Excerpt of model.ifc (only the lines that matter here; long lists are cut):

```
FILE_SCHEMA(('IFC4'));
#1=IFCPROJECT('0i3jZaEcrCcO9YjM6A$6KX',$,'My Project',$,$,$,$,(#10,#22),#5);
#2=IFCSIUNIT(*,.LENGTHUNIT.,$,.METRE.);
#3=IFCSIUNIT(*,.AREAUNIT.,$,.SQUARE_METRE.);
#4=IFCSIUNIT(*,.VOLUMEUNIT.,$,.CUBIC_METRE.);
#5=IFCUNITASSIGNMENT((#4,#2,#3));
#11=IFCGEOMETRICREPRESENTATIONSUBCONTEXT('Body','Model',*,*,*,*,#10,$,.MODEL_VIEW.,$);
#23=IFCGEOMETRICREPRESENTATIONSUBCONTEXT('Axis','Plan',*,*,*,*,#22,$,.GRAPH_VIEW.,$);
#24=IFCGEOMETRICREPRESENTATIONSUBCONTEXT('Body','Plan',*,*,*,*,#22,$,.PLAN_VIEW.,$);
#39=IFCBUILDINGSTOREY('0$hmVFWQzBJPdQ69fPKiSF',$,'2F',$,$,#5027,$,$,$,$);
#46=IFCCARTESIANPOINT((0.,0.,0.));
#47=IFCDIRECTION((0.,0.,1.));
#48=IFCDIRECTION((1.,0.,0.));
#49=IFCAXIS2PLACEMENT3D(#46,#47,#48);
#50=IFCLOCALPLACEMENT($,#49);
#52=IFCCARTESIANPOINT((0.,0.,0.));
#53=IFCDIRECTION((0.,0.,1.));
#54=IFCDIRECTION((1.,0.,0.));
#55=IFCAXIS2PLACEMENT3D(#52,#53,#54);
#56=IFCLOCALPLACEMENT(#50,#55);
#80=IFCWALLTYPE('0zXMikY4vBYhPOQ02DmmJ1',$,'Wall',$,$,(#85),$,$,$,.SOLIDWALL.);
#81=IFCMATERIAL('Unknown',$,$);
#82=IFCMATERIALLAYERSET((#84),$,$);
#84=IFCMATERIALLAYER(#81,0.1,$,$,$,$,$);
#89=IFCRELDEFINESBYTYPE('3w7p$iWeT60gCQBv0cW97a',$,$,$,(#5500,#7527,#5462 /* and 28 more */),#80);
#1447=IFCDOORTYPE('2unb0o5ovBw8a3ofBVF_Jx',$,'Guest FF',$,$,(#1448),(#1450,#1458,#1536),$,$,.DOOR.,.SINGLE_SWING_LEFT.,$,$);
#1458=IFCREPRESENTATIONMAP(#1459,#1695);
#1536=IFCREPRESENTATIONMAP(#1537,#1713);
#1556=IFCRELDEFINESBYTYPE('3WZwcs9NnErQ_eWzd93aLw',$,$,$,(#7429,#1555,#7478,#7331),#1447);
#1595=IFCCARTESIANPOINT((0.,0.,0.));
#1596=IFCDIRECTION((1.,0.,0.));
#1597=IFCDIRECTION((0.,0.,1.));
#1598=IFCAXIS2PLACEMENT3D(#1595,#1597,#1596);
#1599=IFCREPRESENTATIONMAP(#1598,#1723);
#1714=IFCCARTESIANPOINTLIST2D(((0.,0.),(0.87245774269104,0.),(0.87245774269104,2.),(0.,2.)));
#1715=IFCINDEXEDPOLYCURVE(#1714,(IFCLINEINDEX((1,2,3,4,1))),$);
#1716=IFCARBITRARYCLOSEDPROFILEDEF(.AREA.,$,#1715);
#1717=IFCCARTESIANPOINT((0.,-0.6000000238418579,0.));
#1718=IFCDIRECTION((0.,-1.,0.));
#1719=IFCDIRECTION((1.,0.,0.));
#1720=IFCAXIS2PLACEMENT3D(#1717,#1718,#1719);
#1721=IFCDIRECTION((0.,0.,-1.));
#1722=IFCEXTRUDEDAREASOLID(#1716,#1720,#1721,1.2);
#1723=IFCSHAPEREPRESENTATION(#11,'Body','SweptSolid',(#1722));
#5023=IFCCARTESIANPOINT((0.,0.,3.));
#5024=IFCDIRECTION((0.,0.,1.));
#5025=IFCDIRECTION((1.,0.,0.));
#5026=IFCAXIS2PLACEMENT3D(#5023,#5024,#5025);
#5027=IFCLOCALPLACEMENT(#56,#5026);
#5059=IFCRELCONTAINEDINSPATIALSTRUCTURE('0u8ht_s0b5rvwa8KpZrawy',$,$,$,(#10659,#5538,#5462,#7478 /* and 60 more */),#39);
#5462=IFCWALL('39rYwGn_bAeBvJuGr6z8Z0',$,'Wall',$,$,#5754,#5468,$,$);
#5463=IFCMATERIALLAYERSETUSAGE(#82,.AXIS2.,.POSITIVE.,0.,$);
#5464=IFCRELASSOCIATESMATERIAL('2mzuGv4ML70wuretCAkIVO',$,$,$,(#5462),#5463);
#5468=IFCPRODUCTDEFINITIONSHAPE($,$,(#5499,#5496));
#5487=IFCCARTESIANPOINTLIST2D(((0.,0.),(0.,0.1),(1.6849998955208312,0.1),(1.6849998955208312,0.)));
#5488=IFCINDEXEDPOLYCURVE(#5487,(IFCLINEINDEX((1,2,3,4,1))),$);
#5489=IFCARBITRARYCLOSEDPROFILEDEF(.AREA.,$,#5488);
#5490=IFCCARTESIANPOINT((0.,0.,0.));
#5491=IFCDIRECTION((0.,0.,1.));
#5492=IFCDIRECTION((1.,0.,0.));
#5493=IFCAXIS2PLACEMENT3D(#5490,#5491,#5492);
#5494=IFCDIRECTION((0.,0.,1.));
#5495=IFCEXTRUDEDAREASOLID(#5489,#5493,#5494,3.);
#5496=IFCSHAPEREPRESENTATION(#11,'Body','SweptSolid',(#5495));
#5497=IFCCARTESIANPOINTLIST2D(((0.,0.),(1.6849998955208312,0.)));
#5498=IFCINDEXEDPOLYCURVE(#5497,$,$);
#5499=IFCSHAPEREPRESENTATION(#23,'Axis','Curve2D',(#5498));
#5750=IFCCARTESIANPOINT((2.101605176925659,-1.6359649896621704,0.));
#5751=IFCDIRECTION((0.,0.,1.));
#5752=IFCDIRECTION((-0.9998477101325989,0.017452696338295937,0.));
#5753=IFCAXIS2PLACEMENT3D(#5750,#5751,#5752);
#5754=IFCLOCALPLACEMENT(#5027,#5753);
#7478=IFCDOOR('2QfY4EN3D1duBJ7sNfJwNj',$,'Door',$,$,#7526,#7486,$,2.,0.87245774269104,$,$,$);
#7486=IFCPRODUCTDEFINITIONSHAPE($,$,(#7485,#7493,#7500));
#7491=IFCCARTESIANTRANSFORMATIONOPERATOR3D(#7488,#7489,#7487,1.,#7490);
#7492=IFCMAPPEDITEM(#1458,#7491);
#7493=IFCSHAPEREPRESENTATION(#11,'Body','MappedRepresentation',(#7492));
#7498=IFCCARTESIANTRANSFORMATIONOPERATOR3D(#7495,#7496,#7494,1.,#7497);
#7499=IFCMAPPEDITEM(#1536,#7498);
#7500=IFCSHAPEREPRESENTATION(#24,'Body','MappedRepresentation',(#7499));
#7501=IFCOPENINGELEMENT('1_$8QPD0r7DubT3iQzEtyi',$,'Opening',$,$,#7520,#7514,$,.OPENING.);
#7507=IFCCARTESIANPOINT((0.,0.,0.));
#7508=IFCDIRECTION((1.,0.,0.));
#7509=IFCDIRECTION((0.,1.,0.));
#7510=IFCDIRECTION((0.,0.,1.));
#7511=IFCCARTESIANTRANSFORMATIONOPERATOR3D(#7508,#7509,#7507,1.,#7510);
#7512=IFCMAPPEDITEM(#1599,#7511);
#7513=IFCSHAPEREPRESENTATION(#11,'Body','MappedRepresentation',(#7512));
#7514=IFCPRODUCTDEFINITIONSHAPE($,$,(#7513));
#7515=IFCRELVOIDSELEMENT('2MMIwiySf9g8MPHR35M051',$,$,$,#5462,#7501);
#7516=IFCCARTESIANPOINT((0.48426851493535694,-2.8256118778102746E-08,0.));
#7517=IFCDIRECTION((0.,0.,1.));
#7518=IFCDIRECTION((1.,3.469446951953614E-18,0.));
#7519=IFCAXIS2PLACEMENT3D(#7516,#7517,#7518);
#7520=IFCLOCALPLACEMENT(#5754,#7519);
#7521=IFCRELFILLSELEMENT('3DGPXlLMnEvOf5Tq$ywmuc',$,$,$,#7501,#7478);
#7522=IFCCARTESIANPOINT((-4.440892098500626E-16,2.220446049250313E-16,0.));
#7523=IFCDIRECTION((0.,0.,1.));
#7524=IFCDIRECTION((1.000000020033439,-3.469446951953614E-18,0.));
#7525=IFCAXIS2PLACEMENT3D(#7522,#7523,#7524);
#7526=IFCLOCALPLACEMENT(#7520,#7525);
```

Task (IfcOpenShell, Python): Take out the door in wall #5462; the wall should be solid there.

```python
import ifcopenshell
import ifcopenshell.api.feature
import ifcopenshell.api.root
import ifcopenshell.geom
import ifcopenshell.util.shape

model = ifcopenshell.open("model.ifc")
settings = ifcopenshell.geom.settings()


def volume(element):
    """Net volume in cubic metres, openings subtracted."""
    shape = ifcopenshell.geom.create_shape(settings, element)
    return ifcopenshell.util.shape.get_volume(shape.geometry)


door = model.by_id(7478)
opening = door.FillsVoids[0].RelatingOpeningElement
wall = opening.VoidsElements[0].RelatingBuildingElement
before = volume(wall)

ifcopenshell.api.root.remove_product(model, product=door)
ifcopenshell.api.feature.remove_feature(model, feature=opening)

after = volume(wall)

print(f"wall volume {before:.3f} -> {after:.3f} m3")

model.write("model-out.ifc")
```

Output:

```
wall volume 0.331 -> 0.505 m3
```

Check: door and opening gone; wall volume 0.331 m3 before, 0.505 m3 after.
